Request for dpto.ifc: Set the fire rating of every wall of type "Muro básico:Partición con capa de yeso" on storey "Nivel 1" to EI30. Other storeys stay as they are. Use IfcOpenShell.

First a look at what the model holds.

```python
import ifcopenshell
import ifcopenshell.util.element

model = ifcopenshell.open("dpto.ifc")
print(model.schema)
storey = next(s for s in model.by_type("IfcBuildingStorey") if s.Name == "Nivel 1")
walls = [e for e in ifcopenshell.util.element.get_decomposition(storey) if e.is_a("IfcWall")]
seen = {}
for e in walls:
    element_type = ifcopenshell.util.element.get_type(e)
    key = (element_type.Name if element_type != e and element_type else None, ifcopenshell.util.element.get_pset(e, "Pset_WallCommon", "FireRating"))
    seen[key] = seen.get(key, 0) + 1
for (name, value), count in sorted(seen.items(), key=str):
    print(count, "x", name, "|", value)
```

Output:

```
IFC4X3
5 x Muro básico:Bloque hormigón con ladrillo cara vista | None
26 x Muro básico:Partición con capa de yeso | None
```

```python
import ifcopenshell
import ifcopenshell.api.pset
import ifcopenshell.util.element

model = ifcopenshell.open("dpto.ifc")

storey = next(s for s in model.by_type("IfcBuildingStorey") if s.Name == "Nivel 1")
walls = [e for e in ifcopenshell.util.element.get_decomposition(storey) if e.is_a("IfcWall")]

count = 0
for e in walls:
    element_type = ifcopenshell.util.element.get_type(e)
    if element_type in (None, e) or element_type.Name != "Muro básico:Partición con capa de yeso":
        continue
    # add_pset returns the element's existing set when there is one.
    pset = ifcopenshell.api.pset.add_pset(model, product=e, name="Pset_WallCommon")
    ifcopenshell.api.pset.edit_pset(model, pset=pset, properties={"FireRating": "EI30"})
    count += 1

print(count, "walls updated")

model.write("dpto_rev.ifc")
```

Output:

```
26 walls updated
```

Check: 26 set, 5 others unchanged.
